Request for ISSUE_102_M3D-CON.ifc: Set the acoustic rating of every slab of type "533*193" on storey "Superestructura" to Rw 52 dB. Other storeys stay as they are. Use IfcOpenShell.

First a look at what the model holds.

```python
import ifcopenshell
import ifcopenshell.util.element

model = ifcopenshell.open("ISSUE_102_M3D-CON.ifc")
print(model.schema)
storey = next(s for s in model.by_type("IfcBuildingStorey") if s.Name == "Superestructura")
slabs = [e for e in ifcopenshell.util.element.get_decomposition(storey) if e.is_a("IfcSlab")]
seen = {}
for e in slabs:
    element_type = ifcopenshell.util.element.get_type(e)
    key = (element_type.Name if element_type != e and element_type else None, ifcopenshell.util.element.get_pset(e, "Pset_SlabCommon", "AcousticRating"))
    seen[key] = seen.get(key, 0) + 1
for (name, value), count in sorted(seen.items(), key=str):
    print(count, "x", name, "|", value)
```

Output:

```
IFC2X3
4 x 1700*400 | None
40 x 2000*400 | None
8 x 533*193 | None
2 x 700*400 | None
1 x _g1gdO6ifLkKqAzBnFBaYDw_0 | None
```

```python
import ifcopenshell
import ifcopenshell.api.pset
import ifcopenshell.util.element

model = ifcopenshell.open("ISSUE_102_M3D-CON.ifc")

storey = next(s for s in model.by_type("IfcBuildingStorey") if s.Name == "Superestructura")
slabs = [e for e in ifcopenshell.util.element.get_decomposition(storey) if e.is_a("IfcSlab")]

count = 0
for e in slabs:
    element_type = ifcopenshell.util.element.get_type(e)
    if element_type in (None, e) or element_type.Name != "533*193":
        continue
    found = ifcopenshell.util.element.get_pset(e, "Pset_SlabCommon", should_inherit=False)
    if found:
        pset = model.by_id(found["id"])
        if len(ifcopenshell.util.element.get_elements_by_pset(pset)) > 1:
            pset = ifcopenshell.api.pset.unshare_pset(model, products=[e], pset=pset)[0]
    else:
        pset = ifcopenshell.api.pset.add_pset(model, product=e, name="Pset_SlabCommon")
    ifcopenshell.api.pset.edit_pset(model, pset=pset, properties={"AcousticRating": "Rw 52 dB"})
    count += 1

print(count, "slabs updated")

model.write("ISSUE_102_M3D-CON_updated.ifc")
```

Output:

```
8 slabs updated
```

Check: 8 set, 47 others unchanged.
